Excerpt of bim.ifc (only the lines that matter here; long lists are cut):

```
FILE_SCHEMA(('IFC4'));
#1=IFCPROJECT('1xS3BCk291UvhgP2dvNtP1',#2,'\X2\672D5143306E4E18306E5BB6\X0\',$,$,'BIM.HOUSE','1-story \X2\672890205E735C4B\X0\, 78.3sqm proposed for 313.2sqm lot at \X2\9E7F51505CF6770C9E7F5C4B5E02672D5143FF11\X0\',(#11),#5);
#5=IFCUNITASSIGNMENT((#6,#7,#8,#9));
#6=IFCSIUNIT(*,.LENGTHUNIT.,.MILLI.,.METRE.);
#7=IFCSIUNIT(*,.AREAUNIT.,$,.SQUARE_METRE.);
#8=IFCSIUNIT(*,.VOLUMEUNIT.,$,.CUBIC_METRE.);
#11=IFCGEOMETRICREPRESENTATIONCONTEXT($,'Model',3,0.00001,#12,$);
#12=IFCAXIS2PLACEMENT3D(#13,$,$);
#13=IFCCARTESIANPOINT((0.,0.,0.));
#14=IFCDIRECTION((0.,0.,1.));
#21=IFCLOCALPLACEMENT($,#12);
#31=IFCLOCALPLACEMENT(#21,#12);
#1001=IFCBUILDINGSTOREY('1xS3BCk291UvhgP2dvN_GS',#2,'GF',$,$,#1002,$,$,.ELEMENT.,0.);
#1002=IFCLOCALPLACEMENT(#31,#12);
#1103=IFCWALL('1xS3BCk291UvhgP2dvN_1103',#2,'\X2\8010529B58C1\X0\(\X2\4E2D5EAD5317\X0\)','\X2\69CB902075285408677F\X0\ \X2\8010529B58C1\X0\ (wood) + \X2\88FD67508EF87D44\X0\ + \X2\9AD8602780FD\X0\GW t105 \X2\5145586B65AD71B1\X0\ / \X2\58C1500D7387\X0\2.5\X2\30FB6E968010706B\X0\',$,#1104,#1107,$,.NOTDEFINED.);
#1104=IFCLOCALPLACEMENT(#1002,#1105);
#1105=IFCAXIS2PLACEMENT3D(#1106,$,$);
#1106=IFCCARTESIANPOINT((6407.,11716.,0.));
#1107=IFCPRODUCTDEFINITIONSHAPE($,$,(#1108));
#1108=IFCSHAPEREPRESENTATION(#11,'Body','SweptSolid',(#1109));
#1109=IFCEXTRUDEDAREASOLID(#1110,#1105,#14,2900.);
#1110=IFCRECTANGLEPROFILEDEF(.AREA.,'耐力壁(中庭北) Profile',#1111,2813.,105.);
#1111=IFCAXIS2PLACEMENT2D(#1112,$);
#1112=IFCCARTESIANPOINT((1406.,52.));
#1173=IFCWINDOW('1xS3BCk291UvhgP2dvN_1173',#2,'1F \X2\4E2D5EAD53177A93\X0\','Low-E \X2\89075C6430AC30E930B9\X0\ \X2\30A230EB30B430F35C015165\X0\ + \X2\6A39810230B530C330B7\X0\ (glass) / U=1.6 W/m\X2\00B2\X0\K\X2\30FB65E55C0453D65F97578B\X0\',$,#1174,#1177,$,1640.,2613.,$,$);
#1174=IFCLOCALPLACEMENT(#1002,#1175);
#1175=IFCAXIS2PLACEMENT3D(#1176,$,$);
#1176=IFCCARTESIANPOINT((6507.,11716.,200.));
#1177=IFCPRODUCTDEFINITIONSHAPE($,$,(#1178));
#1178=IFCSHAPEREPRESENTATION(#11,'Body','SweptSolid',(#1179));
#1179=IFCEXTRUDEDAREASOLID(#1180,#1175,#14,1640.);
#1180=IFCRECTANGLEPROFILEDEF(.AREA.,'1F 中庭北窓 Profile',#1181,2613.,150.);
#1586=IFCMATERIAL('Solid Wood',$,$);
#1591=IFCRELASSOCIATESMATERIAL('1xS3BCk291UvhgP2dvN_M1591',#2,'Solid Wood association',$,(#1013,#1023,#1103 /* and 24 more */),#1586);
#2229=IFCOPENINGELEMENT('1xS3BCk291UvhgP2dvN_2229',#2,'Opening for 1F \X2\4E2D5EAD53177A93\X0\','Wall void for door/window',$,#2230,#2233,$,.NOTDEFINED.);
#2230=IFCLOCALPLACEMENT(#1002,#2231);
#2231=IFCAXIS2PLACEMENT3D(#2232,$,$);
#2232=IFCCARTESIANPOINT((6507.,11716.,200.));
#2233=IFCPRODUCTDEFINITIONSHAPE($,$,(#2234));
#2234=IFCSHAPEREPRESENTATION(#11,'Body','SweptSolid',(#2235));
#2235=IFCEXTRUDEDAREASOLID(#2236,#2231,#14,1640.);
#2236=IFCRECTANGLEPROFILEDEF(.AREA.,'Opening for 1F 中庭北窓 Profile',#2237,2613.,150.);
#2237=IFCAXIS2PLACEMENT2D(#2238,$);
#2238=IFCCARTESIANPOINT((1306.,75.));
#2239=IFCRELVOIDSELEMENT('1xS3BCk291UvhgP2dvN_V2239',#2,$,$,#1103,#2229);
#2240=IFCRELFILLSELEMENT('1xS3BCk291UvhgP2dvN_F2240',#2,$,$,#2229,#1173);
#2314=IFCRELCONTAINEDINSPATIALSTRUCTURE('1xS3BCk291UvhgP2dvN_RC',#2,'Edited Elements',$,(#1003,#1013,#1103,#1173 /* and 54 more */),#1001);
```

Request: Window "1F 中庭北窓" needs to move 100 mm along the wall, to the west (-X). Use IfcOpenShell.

```python
import ifcopenshell
import ifcopenshell.api.geometry
import ifcopenshell.util.placement
import ifcopenshell.util.unit

model = ifcopenshell.open("bim.ifc")
unit_scale = ifcopenshell.util.unit.calculate_unit_scale(model)

window = model.by_id(1173)
opening = window.FillsVoids[0].RelatingOpeningElement
wall = opening.VoidsElements[0].RelatingBuildingElement

wall_matrix = ifcopenshell.util.placement.get_local_placement(wall.ObjectPlacement)
shift = wall_matrix[:3, 0] * -0.1 / unit_scale
before = ifcopenshell.util.placement.get_local_placement(window.ObjectPlacement)[:3, 3].copy()

# The window is not placed relative to its opening, so move both.
for product in (opening, window):
    matrix = ifcopenshell.util.placement.get_local_placement(product.ObjectPlacement)
    matrix[:3, 3] += shift
    ifcopenshell.api.geometry.edit_object_placement(model, product=product, matrix=matrix, is_si=False)

after = ifcopenshell.util.placement.get_local_placement(window.ObjectPlacement)[:3, 3]
print("window moved by", (after - before).round(3) + 0.0)

model.write("bim_updated.ifc")
```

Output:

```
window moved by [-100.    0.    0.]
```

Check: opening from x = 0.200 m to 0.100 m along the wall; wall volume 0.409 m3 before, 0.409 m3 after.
